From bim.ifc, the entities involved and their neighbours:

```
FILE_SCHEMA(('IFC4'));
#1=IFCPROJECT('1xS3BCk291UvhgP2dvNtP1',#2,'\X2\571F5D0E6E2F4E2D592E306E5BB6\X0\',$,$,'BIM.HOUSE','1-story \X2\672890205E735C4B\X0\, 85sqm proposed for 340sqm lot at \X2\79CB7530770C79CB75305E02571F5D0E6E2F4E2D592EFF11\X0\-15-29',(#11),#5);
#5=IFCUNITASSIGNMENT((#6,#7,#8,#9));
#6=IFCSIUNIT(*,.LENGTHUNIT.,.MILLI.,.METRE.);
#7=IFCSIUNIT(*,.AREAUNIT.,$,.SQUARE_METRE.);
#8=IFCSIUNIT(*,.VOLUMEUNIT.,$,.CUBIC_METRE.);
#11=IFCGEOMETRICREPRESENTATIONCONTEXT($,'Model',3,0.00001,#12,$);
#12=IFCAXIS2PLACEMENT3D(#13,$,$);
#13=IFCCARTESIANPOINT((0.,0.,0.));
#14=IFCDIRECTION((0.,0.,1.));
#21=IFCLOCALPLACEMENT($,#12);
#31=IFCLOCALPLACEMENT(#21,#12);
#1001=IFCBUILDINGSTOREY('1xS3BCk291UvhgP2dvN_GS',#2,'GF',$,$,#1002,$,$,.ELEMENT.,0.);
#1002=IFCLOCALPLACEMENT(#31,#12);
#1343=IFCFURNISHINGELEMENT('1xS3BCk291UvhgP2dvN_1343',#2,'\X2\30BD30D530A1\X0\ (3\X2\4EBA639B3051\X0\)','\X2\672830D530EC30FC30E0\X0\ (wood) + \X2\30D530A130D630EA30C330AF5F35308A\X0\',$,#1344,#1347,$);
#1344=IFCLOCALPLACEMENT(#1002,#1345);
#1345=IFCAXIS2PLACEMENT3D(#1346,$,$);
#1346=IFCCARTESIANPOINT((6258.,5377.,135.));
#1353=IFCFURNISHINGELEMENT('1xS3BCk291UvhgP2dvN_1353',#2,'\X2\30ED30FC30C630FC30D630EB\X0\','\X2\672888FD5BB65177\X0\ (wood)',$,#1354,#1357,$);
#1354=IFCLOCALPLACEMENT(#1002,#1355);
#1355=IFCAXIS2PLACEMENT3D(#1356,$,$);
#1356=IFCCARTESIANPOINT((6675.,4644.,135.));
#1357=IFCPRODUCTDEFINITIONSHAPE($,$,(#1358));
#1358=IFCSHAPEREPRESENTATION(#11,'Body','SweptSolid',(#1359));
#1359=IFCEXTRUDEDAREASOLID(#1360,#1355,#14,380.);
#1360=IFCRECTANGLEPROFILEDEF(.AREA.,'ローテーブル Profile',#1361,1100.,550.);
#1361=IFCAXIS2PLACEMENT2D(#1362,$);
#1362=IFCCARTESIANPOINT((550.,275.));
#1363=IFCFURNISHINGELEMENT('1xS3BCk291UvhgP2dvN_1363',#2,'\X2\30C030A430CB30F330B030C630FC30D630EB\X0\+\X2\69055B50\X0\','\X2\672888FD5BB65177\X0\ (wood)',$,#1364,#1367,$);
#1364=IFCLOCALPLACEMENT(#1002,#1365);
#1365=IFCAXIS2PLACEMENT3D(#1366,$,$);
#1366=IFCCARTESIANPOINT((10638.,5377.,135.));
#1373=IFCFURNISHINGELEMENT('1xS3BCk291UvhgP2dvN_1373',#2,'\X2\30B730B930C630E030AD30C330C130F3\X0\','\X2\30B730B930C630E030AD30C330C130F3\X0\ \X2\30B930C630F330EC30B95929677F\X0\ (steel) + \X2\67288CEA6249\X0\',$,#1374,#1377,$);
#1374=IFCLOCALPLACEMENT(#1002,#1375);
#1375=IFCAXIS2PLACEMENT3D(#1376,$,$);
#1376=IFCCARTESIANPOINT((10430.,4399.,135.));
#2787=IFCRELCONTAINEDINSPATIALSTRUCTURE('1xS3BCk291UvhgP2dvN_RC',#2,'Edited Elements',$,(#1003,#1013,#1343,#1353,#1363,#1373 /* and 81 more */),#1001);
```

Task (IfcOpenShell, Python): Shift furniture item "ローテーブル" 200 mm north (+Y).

```python
import ifcopenshell
import ifcopenshell.api.geometry
import ifcopenshell.util.placement

model = ifcopenshell.open("bim.ifc")

item = model.by_id(1353)
matrix = ifcopenshell.util.placement.get_local_placement(item.ObjectPlacement)
matrix[1, 3] += 200.0
ifcopenshell.api.geometry.edit_object_placement(model, product=item, matrix=matrix, is_si=False)

print(ifcopenshell.util.placement.get_local_placement(item.ObjectPlacement).round(3) + 0.0)

model.write("bim_updated.ifc")
```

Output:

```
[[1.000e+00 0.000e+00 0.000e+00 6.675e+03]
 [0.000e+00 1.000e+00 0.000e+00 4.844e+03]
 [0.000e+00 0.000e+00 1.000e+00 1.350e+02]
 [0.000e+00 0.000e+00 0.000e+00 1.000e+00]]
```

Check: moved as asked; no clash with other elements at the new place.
